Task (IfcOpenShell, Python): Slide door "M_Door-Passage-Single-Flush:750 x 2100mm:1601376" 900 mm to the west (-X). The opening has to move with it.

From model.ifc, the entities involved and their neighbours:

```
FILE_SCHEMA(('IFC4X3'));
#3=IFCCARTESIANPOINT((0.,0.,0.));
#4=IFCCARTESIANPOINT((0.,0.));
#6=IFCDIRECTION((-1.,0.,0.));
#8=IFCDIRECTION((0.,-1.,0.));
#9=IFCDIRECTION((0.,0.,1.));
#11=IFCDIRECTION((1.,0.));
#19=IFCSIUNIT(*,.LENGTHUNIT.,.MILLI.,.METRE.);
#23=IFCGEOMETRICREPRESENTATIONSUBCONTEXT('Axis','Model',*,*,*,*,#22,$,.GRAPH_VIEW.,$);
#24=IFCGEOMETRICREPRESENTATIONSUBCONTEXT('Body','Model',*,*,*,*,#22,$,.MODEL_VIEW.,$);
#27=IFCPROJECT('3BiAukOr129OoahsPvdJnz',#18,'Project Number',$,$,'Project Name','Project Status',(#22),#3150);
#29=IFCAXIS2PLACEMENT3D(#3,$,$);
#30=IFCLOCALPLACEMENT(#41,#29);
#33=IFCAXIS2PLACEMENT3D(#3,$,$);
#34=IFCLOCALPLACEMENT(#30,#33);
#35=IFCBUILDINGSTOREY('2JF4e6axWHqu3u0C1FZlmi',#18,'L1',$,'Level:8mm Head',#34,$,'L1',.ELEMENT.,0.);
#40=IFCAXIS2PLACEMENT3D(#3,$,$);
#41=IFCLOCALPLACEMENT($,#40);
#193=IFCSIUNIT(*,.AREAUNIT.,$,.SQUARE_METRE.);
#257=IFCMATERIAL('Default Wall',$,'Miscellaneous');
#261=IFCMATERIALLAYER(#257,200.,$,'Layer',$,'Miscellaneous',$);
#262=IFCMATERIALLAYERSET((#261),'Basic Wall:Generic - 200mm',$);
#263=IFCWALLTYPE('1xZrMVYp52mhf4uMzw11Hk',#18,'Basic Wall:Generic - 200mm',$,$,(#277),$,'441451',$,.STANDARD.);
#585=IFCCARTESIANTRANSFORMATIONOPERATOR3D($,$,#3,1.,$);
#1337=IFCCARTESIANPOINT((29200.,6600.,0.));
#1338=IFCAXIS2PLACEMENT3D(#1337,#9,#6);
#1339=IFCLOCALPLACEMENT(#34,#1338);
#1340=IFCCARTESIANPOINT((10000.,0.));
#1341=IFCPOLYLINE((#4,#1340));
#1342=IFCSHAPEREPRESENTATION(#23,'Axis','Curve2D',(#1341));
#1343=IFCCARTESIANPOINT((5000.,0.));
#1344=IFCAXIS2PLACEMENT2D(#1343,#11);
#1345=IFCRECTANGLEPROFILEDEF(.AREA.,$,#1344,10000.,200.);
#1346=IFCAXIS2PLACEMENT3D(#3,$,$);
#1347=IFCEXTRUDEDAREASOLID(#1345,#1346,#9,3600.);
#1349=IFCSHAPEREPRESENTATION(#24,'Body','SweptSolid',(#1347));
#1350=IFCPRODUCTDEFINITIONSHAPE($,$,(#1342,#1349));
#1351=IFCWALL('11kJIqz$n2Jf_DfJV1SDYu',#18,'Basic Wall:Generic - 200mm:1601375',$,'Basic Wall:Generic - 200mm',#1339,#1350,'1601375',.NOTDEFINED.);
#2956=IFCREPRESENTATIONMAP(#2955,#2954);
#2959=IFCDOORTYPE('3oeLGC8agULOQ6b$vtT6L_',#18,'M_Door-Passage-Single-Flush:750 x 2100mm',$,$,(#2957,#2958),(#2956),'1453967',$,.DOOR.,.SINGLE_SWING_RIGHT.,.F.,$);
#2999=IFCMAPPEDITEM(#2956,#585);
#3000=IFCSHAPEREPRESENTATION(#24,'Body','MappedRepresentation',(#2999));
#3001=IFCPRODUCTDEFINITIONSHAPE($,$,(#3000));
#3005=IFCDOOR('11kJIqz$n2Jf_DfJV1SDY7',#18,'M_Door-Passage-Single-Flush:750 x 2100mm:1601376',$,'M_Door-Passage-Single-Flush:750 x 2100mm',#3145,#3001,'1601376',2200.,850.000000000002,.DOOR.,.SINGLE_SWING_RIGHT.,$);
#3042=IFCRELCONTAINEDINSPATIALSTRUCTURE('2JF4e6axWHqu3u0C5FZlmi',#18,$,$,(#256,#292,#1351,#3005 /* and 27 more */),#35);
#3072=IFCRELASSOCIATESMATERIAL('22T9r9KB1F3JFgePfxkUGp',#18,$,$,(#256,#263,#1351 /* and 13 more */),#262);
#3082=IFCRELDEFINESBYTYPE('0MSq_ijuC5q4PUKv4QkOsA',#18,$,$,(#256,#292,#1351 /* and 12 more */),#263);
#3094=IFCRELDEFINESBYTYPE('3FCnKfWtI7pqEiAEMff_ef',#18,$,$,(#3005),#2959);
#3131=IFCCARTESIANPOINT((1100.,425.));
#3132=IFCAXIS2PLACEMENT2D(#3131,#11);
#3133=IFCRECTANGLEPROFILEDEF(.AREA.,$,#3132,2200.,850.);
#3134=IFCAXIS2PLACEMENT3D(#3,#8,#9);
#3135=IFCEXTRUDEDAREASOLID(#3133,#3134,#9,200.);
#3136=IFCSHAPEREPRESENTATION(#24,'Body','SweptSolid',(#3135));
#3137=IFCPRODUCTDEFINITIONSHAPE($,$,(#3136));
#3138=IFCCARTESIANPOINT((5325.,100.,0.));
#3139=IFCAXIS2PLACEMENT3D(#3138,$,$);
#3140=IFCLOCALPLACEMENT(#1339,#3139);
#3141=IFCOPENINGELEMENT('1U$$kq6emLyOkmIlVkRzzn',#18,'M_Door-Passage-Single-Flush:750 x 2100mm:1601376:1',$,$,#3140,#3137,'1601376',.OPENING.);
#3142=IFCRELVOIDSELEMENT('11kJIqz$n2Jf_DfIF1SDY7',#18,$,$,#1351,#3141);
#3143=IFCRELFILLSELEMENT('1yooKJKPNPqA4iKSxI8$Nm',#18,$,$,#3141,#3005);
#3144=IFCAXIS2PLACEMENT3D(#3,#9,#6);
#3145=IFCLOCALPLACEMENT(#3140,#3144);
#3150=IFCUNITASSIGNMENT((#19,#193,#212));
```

```python
import ifcopenshell
import ifcopenshell.api.geometry
import ifcopenshell.util.placement
import ifcopenshell.util.unit

model = ifcopenshell.open("model.ifc")
unit_scale = ifcopenshell.util.unit.calculate_unit_scale(model)

door = model.by_guid("11kJIqz$n2Jf_DfJV1SDY7")
opening = door.FillsVoids[0].RelatingOpeningElement
wall = opening.VoidsElements[0].RelatingBuildingElement

wall_matrix = ifcopenshell.util.placement.get_local_placement(wall.ObjectPlacement)
shift = wall_matrix[:3, 0] * 0.9 / unit_scale
before = ifcopenshell.util.placement.get_local_placement(door.ObjectPlacement)[:3, 3].copy()

# The door is placed relative to its opening, so it follows when the opening moves.
matrix = ifcopenshell.util.placement.get_local_placement(opening.ObjectPlacement)
matrix[:3, 3] += shift
ifcopenshell.api.geometry.edit_object_placement(
    model, product=opening, matrix=matrix, is_si=False, should_transform_children=True
)

after = ifcopenshell.util.placement.get_local_placement(door.ObjectPlacement)[:3, 3]
print("door moved by", (after - before).round(3) + 0.0)

model.write("model_updated.ifc")
```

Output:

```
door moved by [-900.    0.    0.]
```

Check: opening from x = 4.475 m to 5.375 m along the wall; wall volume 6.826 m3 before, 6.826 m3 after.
